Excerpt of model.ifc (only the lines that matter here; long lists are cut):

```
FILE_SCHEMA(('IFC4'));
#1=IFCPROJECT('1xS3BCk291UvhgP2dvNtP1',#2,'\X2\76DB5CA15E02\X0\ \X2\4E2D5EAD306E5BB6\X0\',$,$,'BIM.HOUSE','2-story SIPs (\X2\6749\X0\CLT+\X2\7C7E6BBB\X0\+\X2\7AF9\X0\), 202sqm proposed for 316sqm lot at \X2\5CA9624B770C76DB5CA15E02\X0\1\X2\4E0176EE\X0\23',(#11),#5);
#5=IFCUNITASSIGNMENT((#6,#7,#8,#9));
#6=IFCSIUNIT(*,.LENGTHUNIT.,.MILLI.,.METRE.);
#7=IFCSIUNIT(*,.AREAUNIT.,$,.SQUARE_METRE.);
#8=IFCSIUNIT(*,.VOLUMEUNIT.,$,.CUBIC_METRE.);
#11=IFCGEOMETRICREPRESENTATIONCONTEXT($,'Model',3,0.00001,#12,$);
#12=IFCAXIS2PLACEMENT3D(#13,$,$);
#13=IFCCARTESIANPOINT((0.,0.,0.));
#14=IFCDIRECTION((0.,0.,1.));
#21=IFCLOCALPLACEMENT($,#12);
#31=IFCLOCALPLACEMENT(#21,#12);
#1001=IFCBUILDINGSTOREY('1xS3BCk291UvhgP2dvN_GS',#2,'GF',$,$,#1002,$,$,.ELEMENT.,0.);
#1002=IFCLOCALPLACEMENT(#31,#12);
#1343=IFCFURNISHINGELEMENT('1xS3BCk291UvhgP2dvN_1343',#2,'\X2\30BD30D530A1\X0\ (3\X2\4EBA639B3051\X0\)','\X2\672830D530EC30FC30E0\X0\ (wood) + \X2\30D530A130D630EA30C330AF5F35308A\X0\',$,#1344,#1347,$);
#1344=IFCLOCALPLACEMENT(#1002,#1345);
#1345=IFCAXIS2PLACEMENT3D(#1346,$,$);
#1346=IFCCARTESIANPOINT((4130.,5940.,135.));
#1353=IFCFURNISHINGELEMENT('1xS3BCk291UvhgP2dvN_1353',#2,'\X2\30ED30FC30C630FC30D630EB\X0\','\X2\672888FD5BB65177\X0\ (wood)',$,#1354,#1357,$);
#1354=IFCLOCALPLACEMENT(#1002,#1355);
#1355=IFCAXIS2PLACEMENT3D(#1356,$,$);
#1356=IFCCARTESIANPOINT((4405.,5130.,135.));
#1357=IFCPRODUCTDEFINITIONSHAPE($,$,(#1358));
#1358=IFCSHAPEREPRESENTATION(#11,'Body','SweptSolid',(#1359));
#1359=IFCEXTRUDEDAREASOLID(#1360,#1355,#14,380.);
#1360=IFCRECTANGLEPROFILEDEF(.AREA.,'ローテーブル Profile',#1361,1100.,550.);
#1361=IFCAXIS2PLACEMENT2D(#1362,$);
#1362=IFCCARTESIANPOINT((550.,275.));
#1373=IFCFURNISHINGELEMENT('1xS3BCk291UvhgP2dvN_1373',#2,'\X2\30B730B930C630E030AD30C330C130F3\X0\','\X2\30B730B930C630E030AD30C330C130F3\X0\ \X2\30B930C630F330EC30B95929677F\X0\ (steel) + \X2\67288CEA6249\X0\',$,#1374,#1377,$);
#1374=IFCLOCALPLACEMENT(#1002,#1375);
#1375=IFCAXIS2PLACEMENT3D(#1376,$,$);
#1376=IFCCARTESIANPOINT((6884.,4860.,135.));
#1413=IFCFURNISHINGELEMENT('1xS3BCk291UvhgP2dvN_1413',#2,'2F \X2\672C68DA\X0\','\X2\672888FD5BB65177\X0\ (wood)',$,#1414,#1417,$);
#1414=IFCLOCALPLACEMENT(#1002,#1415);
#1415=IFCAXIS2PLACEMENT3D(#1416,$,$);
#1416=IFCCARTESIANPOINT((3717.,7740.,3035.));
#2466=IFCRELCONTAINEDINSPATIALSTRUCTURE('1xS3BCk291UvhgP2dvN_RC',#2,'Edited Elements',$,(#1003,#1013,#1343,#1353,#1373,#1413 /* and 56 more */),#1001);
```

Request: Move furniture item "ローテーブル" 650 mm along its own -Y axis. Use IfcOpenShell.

```python
import ifcopenshell
import ifcopenshell.api.geometry
import ifcopenshell.util.placement

model = ifcopenshell.open("model.ifc")

item = model.by_id(1353)
matrix = ifcopenshell.util.placement.get_local_placement(item.ObjectPlacement)
matrix[:3, 3] -= matrix[:3, 1] * 650.0
ifcopenshell.api.geometry.edit_object_placement(model, product=item, matrix=matrix, is_si=False)

print(ifcopenshell.util.placement.get_local_placement(item.ObjectPlacement).round(3) + 0.0)

model.write("model_edited.ifc")
```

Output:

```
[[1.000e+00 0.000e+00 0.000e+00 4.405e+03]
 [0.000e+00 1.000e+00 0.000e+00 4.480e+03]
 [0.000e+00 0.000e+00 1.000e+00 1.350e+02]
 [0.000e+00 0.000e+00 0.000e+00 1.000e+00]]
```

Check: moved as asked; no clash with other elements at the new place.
